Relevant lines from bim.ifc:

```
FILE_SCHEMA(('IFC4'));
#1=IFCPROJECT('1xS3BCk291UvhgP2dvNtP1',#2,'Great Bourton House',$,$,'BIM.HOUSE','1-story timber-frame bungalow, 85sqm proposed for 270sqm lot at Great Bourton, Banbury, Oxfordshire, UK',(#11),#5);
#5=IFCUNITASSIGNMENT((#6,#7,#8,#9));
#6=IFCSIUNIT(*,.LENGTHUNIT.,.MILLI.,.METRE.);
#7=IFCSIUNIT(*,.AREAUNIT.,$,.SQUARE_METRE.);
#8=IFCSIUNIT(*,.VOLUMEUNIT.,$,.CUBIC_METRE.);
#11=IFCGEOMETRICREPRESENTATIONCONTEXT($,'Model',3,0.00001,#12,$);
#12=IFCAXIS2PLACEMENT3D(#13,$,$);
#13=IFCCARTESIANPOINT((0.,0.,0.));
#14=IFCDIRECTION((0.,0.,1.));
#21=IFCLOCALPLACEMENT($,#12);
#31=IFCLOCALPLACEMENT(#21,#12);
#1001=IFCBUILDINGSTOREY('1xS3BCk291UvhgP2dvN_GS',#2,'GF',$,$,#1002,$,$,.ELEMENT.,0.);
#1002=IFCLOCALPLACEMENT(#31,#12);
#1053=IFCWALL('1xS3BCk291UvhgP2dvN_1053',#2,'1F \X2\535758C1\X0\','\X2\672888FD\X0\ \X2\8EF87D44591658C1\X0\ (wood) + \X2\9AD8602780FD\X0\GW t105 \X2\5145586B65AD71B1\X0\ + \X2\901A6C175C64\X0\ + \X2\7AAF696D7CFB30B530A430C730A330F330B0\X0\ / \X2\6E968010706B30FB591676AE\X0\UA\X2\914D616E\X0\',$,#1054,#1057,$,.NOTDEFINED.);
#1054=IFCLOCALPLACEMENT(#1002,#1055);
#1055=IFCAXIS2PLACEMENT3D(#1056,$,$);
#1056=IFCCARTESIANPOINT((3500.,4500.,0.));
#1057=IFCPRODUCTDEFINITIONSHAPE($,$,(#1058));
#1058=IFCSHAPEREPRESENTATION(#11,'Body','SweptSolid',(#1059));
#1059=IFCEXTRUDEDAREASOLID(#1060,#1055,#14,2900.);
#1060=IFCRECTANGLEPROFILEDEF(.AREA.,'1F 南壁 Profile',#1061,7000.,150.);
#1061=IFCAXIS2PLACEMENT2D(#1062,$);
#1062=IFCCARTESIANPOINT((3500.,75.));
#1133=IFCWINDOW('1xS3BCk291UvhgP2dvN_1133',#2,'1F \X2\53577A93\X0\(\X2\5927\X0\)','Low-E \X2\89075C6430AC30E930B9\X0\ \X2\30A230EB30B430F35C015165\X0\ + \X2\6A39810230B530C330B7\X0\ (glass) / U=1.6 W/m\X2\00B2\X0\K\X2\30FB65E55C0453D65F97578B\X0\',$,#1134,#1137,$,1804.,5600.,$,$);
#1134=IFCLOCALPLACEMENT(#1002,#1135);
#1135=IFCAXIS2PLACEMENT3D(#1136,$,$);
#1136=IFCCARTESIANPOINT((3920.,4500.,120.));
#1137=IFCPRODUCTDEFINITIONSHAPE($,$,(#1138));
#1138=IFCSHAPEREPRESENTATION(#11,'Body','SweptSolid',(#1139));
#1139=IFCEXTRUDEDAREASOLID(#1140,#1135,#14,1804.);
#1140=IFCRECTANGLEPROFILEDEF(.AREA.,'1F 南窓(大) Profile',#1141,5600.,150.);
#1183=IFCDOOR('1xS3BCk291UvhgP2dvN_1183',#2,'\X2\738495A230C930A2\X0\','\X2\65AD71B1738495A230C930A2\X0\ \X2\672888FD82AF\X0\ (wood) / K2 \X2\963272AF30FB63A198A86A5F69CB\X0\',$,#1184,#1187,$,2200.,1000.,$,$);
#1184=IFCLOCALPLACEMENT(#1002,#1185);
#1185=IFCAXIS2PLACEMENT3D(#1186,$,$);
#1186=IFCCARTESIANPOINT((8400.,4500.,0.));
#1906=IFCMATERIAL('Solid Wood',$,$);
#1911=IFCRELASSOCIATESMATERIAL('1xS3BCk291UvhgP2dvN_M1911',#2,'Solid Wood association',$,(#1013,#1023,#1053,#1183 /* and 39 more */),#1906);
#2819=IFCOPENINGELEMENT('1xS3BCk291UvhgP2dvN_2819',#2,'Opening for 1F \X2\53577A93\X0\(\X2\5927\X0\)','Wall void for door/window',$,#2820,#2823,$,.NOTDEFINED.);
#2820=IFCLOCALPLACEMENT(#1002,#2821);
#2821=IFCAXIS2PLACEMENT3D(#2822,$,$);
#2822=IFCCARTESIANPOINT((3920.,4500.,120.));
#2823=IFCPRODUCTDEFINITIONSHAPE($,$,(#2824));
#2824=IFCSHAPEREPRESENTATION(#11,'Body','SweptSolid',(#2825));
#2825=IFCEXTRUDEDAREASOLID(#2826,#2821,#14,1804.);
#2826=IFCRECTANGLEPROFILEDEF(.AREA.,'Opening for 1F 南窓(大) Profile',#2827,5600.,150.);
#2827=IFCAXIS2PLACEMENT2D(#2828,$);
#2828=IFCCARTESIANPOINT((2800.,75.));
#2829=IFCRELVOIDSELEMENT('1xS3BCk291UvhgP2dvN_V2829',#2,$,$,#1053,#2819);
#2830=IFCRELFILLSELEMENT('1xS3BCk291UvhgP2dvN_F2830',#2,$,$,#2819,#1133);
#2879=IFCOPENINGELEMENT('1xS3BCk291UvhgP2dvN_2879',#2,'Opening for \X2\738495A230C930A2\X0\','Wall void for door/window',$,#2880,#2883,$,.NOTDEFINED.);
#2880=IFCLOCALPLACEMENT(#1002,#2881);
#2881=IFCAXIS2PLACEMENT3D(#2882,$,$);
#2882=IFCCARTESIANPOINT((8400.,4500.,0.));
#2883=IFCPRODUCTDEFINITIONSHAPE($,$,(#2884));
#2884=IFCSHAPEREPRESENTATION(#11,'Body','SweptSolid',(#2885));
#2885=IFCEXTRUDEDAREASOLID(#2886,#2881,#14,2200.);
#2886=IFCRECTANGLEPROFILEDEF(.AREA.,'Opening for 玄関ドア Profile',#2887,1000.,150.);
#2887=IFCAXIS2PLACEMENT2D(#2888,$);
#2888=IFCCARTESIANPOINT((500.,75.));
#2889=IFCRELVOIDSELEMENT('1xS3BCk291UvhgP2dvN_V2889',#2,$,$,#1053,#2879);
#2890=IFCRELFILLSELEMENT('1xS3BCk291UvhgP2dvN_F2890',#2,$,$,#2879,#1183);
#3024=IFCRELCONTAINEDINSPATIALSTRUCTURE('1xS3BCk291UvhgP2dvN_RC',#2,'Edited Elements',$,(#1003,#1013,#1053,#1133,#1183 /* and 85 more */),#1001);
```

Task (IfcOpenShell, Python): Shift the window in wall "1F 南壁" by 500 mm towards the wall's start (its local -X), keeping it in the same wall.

```python
import ifcopenshell
import ifcopenshell.api.geometry
import ifcopenshell.util.placement
import ifcopenshell.util.unit

model = ifcopenshell.open("bim.ifc")
unit_scale = ifcopenshell.util.unit.calculate_unit_scale(model)

window = model.by_id(1133)
opening = window.FillsVoids[0].RelatingOpeningElement
wall = opening.VoidsElements[0].RelatingBuildingElement

wall_matrix = ifcopenshell.util.placement.get_local_placement(wall.ObjectPlacement)
shift = wall_matrix[:3, 0] * -0.5 / unit_scale
before = ifcopenshell.util.placement.get_local_placement(window.ObjectPlacement)[:3, 3].copy()

# The window is not placed relative to its opening, so move both.
for product in (opening, window):
    matrix = ifcopenshell.util.placement.get_local_placement(product.ObjectPlacement)
    matrix[:3, 3] += shift
    ifcopenshell.api.geometry.edit_object_placement(model, product=product, matrix=matrix, is_si=False)

after = ifcopenshell.util.placement.get_local_placement(window.ObjectPlacement)[:3, 3]
print("window moved by", (after - before).round(3) + 0.0)

model.write("bim_edited.ifc")
```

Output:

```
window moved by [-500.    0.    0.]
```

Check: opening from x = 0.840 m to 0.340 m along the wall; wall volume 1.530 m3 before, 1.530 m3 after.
